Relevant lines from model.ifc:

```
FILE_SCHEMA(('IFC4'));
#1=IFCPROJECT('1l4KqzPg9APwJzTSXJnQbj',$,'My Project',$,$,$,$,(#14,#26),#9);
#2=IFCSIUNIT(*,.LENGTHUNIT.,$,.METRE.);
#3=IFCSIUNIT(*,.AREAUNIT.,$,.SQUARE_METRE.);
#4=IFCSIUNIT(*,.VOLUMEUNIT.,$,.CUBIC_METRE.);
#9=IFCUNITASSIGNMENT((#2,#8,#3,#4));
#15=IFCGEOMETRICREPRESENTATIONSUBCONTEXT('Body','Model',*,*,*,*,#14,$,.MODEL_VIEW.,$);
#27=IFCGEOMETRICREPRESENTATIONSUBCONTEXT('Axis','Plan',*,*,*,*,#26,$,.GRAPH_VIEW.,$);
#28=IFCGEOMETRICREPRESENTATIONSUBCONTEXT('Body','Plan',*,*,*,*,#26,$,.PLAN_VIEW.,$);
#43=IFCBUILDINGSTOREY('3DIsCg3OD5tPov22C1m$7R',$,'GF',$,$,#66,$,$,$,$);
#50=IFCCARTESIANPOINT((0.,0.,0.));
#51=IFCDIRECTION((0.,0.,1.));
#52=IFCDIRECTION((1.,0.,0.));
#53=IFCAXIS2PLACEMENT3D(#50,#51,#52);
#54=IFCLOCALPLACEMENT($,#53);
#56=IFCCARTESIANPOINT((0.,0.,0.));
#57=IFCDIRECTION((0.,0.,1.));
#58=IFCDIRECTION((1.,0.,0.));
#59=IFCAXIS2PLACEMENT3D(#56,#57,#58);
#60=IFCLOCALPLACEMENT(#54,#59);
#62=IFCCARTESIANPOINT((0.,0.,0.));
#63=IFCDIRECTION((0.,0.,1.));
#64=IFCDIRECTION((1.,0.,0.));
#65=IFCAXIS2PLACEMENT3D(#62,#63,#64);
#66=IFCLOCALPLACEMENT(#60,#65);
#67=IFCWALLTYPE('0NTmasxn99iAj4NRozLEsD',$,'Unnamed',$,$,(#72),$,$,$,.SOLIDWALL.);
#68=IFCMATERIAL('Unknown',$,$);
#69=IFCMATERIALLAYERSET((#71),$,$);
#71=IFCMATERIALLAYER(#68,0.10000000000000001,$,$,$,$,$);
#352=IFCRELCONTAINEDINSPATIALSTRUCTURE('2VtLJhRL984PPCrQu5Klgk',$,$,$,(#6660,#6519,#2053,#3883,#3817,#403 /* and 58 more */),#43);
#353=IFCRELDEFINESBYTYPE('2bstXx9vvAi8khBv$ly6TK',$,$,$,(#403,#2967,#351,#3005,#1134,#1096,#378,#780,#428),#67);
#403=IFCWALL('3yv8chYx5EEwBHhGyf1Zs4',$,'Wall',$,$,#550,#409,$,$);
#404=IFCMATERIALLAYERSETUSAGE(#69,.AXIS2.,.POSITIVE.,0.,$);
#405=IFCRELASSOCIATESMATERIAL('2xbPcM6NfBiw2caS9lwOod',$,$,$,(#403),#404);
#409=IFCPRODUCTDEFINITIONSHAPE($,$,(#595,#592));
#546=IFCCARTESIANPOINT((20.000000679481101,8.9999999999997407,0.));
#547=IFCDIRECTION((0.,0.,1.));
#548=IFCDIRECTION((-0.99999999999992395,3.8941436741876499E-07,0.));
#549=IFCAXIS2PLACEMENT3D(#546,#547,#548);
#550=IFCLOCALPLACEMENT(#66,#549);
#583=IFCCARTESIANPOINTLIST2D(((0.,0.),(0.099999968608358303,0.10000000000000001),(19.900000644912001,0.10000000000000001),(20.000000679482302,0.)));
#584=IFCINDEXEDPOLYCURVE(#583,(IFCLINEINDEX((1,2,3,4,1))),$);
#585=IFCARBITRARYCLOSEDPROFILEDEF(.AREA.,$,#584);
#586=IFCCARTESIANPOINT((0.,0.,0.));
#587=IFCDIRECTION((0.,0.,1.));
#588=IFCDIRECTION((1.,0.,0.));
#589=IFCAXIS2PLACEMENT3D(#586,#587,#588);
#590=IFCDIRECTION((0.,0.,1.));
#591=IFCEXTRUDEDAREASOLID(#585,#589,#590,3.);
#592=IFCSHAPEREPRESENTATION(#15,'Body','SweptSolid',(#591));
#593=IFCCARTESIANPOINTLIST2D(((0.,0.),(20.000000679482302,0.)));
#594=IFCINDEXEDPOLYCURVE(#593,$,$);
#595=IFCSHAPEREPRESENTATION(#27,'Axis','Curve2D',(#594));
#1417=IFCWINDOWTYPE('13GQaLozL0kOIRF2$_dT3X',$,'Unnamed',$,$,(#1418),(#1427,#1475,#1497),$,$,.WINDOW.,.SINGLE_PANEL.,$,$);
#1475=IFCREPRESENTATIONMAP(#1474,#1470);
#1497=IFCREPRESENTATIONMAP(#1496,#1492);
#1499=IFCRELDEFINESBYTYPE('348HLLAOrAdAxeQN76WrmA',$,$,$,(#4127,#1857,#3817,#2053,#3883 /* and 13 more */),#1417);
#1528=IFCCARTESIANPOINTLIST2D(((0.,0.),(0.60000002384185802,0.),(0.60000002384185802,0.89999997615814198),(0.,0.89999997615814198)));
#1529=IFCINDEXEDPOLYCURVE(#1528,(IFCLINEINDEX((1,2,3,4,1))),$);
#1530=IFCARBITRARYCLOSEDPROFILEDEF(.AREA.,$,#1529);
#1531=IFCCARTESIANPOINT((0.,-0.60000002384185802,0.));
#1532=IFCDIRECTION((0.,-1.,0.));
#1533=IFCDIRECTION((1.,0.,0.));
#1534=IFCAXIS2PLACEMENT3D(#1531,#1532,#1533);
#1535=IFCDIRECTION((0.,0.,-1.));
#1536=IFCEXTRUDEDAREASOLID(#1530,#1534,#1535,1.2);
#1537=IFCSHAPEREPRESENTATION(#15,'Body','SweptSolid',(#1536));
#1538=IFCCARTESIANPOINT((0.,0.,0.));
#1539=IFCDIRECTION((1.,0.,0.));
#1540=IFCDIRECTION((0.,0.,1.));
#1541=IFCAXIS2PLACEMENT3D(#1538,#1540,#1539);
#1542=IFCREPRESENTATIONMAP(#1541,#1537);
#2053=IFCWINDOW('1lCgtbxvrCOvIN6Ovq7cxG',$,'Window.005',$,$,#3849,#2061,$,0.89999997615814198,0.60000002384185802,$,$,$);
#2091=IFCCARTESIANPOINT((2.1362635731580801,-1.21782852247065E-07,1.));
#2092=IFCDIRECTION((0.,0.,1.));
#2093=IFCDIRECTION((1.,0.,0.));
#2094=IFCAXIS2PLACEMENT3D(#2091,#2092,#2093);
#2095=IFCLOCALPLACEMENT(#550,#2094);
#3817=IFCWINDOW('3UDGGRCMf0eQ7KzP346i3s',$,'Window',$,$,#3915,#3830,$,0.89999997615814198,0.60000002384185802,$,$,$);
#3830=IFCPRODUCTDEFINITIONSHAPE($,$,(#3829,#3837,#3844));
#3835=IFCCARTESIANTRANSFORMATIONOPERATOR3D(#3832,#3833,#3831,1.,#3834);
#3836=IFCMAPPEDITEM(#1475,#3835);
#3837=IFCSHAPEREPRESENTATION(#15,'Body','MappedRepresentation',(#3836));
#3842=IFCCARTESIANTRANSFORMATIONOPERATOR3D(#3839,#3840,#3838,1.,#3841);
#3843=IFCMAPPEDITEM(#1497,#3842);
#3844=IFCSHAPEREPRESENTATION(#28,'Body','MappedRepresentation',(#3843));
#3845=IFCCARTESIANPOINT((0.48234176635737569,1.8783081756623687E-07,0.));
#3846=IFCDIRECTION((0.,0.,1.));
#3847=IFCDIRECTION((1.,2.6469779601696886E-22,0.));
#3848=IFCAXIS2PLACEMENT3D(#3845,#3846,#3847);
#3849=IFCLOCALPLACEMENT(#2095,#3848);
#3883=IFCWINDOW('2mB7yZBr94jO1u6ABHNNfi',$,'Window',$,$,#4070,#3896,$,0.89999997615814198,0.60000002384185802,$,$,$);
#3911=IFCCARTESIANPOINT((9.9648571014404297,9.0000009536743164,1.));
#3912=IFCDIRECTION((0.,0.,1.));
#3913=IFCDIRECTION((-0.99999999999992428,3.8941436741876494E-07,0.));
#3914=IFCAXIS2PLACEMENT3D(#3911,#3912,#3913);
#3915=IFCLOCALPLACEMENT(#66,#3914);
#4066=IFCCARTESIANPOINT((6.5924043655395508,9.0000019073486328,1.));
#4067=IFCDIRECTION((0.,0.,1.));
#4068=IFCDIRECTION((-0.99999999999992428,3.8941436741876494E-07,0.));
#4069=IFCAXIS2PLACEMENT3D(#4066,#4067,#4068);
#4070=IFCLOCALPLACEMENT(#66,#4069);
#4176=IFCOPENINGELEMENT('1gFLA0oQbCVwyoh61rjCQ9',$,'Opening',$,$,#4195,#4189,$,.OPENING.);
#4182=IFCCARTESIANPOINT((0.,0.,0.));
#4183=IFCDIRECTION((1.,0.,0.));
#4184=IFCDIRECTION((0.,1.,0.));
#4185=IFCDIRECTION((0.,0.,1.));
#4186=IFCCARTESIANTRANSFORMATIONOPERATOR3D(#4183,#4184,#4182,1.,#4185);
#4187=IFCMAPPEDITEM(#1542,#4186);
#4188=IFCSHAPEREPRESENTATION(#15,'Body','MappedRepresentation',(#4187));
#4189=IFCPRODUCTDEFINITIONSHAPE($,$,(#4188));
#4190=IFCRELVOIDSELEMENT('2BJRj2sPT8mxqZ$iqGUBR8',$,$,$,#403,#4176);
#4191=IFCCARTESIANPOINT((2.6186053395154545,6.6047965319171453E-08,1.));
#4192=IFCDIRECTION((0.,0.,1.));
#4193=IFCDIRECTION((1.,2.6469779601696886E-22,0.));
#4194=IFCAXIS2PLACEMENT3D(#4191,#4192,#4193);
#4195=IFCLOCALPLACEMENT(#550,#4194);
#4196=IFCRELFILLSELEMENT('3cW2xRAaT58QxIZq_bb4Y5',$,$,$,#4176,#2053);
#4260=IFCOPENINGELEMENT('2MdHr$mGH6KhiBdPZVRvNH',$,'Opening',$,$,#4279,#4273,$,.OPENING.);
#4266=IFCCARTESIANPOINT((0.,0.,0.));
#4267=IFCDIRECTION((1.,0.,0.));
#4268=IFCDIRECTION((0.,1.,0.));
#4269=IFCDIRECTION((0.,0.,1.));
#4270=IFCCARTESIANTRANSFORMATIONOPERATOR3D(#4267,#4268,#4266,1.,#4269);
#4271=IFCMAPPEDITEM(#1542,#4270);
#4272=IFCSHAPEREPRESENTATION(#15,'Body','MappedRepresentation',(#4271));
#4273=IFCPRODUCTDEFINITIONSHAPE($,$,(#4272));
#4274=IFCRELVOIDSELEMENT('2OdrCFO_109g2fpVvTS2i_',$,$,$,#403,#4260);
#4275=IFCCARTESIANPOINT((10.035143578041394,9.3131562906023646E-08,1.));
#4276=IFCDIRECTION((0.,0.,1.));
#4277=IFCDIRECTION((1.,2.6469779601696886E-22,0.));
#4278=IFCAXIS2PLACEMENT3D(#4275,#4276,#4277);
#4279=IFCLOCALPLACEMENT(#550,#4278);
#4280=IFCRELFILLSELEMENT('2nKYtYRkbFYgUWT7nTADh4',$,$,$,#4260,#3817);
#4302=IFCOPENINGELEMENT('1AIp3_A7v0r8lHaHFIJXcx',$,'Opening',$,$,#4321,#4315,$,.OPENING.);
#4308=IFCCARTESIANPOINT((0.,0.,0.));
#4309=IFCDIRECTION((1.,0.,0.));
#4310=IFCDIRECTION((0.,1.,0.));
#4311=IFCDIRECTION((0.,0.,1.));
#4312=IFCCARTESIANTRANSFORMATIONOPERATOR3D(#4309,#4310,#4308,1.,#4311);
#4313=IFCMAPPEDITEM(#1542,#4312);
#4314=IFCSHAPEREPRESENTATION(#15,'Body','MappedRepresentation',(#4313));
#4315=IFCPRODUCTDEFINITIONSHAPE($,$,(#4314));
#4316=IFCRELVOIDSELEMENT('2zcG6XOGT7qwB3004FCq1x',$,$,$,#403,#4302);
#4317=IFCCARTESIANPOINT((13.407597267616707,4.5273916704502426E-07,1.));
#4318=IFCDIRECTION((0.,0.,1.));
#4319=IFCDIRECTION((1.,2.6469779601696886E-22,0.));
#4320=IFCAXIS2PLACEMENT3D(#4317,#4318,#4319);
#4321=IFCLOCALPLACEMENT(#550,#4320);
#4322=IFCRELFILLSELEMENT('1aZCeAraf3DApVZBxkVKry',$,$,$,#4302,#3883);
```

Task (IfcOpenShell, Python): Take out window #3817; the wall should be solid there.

```python
import ifcopenshell
import ifcopenshell.api.feature
import ifcopenshell.api.root
import ifcopenshell.geom
import ifcopenshell.util.shape

model = ifcopenshell.open("model.ifc")
settings = ifcopenshell.geom.settings()


def volume(element):
    """Net volume in cubic metres, openings subtracted."""
    shape = ifcopenshell.geom.create_shape(settings, element)
    return ifcopenshell.util.shape.get_volume(shape.geometry)


window = model.by_id(3817)
opening = window.FillsVoids[0].RelatingOpeningElement
wall = opening.VoidsElements[0].RelatingBuildingElement
before = volume(wall)

ifcopenshell.api.root.remove_product(model, product=window)
ifcopenshell.api.feature.remove_feature(model, feature=opening)

after = volume(wall)

print(f"wall volume {before:.3f} -> {after:.3f} m3")

model.write("model_edited.ifc")
```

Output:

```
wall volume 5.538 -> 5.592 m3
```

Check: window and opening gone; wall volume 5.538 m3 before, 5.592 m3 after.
